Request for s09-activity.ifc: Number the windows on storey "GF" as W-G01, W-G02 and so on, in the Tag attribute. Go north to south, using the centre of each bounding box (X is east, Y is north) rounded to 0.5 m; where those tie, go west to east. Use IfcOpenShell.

First a look at what the model holds.

```python
import ifcopenshell
import ifcopenshell.util.element
import ifcopenshell.util.placement

model = ifcopenshell.open("s09-activity.ifc")
print(model.schema)
storey = next(s for s in model.by_type("IfcBuildingStorey") if s.Name == "GF")
windows = [e for e in ifcopenshell.util.element.get_decomposition(storey) if e.is_a("IfcWindow")]
for e in sorted(windows, key=lambda e: e.id()):
    origin = ifcopenshell.util.placement.get_local_placement(e.ObjectPlacement)[:3, 3]
    print(e.id(), e.Tag, e.Name, origin.round(2) + 0.0, sep=" | ")
```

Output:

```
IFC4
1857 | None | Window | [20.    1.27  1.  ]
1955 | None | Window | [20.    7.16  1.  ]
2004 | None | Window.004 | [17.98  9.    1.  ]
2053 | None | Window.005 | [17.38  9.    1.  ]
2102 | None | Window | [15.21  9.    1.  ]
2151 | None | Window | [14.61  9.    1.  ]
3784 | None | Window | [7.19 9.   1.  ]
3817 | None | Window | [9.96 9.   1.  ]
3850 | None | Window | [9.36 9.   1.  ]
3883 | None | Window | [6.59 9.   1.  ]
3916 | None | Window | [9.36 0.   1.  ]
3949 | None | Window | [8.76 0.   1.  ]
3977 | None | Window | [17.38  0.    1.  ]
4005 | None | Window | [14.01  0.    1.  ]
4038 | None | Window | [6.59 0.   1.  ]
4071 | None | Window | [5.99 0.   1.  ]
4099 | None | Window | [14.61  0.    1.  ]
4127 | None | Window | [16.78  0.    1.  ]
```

```python
import ifcopenshell
import ifcopenshell.geom
import ifcopenshell.util.element
import ifcopenshell.util.shape

model = ifcopenshell.open("s09-activity.ifc")
settings = ifcopenshell.geom.settings()
settings.set("use-world-coords", True)


def centre(element):
    shape = ifcopenshell.geom.create_shape(settings, element)
    return ifcopenshell.util.shape.get_bbox_centroid(shape.geometry)


storey = next(s for s in model.by_type("IfcBuildingStorey") if s.Name == "GF")
windows = [e for e in ifcopenshell.util.element.get_decomposition(storey) if e.is_a("IfcWindow")]

# Insertion points can sit at a corner or the storey origin, so sort by the geometry (in metres).
centres = {e: centre(e) for e in windows}
windows.sort(key=lambda e: (-round(centres[e][1] / 0.5), centres[e][0]))

for i, e in enumerate(windows, start=1):
    number = f"W-G{i:02d}"
    e.Tag = number
    print(e.id(), number)

model.write("s09-activity_edited.ifc")
```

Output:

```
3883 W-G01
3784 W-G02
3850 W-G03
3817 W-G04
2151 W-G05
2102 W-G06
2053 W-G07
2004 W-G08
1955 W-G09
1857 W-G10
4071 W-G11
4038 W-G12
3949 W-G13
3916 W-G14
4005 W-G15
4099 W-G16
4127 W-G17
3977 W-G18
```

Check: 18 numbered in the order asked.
